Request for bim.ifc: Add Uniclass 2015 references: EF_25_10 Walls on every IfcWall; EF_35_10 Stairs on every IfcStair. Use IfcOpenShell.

First a look at what the model holds.

```python
import ifcopenshell

model = ifcopenshell.open("bim.ifc")
print(model.schema)
print("classifications:", [c.Name for c in model.by_type("IfcClassification")])
for ifc_class in ("IfcDoor", "IfcRoof", "IfcStair", "IfcWall", "IfcWindow"):
    print(ifc_class, len(model.by_type(ifc_class)))
```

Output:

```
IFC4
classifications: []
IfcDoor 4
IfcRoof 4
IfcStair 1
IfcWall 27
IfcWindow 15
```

```python
import ifcopenshell
import ifcopenshell.api.classification

model = ifcopenshell.open("bim.ifc")

system = ifcopenshell.api.classification.add_classification(model, classification="Uniclass 2015")

codes = {
    "IfcWall": ("EF_25_10", "Walls"),
    "IfcStair": ("EF_35_10", "Stairs"),
}
for ifc_class, (code, name) in codes.items():
    products = model.by_type(ifc_class)
    ifcopenshell.api.classification.add_reference(
        model, products=products, classification=system, identification=code, name=name
    )
    print(code, len(products))

model.write("bim_v2.ifc")
```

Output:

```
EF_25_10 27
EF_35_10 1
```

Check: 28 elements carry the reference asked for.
